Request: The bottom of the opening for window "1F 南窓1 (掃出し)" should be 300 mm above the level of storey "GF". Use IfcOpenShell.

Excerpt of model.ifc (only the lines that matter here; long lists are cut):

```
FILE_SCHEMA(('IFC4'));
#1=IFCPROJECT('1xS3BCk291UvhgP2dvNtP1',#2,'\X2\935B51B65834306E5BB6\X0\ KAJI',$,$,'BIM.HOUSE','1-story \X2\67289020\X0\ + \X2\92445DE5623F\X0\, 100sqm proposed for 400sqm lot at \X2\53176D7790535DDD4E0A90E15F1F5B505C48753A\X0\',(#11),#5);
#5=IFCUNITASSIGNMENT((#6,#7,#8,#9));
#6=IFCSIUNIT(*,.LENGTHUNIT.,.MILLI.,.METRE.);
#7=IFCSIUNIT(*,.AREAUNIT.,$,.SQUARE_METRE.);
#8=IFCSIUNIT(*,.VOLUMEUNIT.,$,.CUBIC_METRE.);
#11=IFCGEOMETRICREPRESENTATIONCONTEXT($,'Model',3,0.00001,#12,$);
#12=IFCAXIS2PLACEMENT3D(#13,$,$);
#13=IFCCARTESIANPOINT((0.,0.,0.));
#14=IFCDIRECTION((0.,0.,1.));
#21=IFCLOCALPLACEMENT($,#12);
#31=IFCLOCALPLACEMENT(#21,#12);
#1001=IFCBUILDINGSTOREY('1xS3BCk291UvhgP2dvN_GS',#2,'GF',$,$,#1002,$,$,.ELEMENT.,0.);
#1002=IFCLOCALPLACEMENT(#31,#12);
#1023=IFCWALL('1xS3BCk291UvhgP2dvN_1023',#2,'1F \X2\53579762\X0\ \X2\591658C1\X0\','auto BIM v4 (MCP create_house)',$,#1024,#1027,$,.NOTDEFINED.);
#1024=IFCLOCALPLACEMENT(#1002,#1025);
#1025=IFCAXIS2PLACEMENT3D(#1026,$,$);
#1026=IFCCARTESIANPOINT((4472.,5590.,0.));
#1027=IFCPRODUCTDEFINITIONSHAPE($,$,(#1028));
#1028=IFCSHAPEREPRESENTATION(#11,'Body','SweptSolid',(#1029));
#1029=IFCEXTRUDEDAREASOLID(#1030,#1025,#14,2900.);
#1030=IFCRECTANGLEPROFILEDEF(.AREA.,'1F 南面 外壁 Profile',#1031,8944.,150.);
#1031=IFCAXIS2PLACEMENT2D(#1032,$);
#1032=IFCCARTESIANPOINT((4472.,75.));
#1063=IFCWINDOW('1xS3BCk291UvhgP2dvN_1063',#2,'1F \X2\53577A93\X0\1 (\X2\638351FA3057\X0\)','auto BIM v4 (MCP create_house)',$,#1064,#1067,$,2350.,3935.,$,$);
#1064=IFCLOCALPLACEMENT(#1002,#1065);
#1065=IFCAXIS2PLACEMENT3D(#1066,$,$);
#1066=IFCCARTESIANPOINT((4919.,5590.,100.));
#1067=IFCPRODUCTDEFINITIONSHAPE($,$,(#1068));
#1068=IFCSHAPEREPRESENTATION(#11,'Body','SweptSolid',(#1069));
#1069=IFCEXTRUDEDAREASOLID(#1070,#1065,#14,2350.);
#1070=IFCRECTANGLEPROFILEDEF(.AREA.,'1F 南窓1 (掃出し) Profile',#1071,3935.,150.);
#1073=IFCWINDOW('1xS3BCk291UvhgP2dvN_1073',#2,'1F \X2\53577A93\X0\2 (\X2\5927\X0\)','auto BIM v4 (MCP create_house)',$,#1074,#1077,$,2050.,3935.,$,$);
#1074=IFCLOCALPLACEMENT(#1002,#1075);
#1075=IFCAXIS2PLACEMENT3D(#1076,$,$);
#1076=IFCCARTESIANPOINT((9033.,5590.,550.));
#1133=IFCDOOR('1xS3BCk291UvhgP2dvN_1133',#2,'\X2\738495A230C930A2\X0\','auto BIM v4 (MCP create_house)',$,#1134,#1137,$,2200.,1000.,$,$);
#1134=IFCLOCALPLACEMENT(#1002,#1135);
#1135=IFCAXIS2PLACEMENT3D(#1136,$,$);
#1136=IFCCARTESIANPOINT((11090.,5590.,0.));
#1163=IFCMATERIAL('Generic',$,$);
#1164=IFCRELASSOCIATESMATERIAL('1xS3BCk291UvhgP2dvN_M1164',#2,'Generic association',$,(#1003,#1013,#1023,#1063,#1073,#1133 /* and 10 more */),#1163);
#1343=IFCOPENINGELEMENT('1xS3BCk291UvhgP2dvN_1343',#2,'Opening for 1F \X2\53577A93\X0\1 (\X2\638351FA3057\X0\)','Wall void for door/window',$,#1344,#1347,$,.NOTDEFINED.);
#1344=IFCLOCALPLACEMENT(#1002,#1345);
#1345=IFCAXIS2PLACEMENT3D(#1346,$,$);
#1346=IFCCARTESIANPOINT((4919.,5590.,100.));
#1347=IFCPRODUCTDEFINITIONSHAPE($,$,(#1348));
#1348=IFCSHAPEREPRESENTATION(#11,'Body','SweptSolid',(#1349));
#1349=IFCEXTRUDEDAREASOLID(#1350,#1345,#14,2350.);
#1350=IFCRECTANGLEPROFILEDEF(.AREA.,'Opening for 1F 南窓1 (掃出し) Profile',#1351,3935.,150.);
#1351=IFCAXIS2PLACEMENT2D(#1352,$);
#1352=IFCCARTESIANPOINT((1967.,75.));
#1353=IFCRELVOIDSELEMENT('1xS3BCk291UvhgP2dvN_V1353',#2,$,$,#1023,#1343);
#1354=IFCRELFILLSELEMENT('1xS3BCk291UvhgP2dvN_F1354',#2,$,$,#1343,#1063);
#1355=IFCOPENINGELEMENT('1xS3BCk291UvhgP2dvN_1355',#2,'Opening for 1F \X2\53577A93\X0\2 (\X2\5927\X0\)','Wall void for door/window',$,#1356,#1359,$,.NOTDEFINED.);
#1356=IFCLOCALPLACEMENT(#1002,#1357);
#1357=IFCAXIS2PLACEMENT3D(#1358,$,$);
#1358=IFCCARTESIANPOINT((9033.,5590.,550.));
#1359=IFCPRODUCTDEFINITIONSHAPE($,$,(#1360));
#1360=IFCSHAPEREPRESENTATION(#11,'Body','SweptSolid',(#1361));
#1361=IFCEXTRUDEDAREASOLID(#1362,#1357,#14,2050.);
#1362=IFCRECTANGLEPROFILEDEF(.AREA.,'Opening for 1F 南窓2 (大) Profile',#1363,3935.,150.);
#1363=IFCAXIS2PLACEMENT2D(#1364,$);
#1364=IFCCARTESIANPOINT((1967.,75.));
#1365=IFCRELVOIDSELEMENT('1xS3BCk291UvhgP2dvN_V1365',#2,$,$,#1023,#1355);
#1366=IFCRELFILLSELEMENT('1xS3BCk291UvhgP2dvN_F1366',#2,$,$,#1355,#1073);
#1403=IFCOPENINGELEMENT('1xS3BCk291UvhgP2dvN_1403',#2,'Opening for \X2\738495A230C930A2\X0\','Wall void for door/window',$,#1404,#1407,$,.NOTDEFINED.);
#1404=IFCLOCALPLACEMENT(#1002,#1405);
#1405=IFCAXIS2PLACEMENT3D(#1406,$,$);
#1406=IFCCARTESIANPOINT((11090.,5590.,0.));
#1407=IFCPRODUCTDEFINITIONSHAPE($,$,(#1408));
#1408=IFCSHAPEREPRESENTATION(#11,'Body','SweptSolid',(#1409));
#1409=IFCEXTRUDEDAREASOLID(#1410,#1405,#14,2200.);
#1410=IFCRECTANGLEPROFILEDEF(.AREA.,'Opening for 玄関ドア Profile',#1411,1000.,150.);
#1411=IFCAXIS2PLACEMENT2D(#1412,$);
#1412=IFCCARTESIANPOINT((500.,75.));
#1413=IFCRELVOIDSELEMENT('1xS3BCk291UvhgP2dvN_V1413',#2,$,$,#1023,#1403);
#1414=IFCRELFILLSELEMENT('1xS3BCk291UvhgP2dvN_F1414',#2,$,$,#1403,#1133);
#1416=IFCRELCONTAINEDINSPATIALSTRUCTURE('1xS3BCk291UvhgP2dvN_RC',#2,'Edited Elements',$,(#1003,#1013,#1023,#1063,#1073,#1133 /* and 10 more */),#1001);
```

```python
import numpy as np
import ifcopenshell
import ifcopenshell.api.geometry
import ifcopenshell.geom
import ifcopenshell.util.element
import ifcopenshell.util.placement
import ifcopenshell.util.shape
import ifcopenshell.util.unit

model = ifcopenshell.open("model.ifc")
unit_scale = ifcopenshell.util.unit.calculate_unit_scale(model)

window = model.by_id(1063)
opening = window.FillsVoids[0].RelatingOpeningElement
storey = ifcopenshell.util.element.get_container(window, ifc_class="IfcBuildingStorey")
level = ifcopenshell.util.placement.get_local_placement(storey.ObjectPlacement)[2, 3]

# The opening's origin need not be at the sill, so measure its lowest point.
shape = ifcopenshell.geom.create_shape(ifcopenshell.geom.settings(), opening)
bottom = ifcopenshell.util.shape.get_shape_bottom_elevation(shape, shape.geometry) / unit_scale
dz = level + 0.3 / unit_scale - bottom

shift = np.array([0.0, 0.0, dz])
# The window is not placed relative to its opening, so move both.
for product in (opening, window):
    matrix = ifcopenshell.util.placement.get_local_placement(product.ObjectPlacement)
    matrix[:3, 3] += shift
    ifcopenshell.api.geometry.edit_object_placement(model, product=product, matrix=matrix, is_si=False)

print(f"moved by {dz * unit_scale:+.3f} m")

model.write("model_edited.ifc")
```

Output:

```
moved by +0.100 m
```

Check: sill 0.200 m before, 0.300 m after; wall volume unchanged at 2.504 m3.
